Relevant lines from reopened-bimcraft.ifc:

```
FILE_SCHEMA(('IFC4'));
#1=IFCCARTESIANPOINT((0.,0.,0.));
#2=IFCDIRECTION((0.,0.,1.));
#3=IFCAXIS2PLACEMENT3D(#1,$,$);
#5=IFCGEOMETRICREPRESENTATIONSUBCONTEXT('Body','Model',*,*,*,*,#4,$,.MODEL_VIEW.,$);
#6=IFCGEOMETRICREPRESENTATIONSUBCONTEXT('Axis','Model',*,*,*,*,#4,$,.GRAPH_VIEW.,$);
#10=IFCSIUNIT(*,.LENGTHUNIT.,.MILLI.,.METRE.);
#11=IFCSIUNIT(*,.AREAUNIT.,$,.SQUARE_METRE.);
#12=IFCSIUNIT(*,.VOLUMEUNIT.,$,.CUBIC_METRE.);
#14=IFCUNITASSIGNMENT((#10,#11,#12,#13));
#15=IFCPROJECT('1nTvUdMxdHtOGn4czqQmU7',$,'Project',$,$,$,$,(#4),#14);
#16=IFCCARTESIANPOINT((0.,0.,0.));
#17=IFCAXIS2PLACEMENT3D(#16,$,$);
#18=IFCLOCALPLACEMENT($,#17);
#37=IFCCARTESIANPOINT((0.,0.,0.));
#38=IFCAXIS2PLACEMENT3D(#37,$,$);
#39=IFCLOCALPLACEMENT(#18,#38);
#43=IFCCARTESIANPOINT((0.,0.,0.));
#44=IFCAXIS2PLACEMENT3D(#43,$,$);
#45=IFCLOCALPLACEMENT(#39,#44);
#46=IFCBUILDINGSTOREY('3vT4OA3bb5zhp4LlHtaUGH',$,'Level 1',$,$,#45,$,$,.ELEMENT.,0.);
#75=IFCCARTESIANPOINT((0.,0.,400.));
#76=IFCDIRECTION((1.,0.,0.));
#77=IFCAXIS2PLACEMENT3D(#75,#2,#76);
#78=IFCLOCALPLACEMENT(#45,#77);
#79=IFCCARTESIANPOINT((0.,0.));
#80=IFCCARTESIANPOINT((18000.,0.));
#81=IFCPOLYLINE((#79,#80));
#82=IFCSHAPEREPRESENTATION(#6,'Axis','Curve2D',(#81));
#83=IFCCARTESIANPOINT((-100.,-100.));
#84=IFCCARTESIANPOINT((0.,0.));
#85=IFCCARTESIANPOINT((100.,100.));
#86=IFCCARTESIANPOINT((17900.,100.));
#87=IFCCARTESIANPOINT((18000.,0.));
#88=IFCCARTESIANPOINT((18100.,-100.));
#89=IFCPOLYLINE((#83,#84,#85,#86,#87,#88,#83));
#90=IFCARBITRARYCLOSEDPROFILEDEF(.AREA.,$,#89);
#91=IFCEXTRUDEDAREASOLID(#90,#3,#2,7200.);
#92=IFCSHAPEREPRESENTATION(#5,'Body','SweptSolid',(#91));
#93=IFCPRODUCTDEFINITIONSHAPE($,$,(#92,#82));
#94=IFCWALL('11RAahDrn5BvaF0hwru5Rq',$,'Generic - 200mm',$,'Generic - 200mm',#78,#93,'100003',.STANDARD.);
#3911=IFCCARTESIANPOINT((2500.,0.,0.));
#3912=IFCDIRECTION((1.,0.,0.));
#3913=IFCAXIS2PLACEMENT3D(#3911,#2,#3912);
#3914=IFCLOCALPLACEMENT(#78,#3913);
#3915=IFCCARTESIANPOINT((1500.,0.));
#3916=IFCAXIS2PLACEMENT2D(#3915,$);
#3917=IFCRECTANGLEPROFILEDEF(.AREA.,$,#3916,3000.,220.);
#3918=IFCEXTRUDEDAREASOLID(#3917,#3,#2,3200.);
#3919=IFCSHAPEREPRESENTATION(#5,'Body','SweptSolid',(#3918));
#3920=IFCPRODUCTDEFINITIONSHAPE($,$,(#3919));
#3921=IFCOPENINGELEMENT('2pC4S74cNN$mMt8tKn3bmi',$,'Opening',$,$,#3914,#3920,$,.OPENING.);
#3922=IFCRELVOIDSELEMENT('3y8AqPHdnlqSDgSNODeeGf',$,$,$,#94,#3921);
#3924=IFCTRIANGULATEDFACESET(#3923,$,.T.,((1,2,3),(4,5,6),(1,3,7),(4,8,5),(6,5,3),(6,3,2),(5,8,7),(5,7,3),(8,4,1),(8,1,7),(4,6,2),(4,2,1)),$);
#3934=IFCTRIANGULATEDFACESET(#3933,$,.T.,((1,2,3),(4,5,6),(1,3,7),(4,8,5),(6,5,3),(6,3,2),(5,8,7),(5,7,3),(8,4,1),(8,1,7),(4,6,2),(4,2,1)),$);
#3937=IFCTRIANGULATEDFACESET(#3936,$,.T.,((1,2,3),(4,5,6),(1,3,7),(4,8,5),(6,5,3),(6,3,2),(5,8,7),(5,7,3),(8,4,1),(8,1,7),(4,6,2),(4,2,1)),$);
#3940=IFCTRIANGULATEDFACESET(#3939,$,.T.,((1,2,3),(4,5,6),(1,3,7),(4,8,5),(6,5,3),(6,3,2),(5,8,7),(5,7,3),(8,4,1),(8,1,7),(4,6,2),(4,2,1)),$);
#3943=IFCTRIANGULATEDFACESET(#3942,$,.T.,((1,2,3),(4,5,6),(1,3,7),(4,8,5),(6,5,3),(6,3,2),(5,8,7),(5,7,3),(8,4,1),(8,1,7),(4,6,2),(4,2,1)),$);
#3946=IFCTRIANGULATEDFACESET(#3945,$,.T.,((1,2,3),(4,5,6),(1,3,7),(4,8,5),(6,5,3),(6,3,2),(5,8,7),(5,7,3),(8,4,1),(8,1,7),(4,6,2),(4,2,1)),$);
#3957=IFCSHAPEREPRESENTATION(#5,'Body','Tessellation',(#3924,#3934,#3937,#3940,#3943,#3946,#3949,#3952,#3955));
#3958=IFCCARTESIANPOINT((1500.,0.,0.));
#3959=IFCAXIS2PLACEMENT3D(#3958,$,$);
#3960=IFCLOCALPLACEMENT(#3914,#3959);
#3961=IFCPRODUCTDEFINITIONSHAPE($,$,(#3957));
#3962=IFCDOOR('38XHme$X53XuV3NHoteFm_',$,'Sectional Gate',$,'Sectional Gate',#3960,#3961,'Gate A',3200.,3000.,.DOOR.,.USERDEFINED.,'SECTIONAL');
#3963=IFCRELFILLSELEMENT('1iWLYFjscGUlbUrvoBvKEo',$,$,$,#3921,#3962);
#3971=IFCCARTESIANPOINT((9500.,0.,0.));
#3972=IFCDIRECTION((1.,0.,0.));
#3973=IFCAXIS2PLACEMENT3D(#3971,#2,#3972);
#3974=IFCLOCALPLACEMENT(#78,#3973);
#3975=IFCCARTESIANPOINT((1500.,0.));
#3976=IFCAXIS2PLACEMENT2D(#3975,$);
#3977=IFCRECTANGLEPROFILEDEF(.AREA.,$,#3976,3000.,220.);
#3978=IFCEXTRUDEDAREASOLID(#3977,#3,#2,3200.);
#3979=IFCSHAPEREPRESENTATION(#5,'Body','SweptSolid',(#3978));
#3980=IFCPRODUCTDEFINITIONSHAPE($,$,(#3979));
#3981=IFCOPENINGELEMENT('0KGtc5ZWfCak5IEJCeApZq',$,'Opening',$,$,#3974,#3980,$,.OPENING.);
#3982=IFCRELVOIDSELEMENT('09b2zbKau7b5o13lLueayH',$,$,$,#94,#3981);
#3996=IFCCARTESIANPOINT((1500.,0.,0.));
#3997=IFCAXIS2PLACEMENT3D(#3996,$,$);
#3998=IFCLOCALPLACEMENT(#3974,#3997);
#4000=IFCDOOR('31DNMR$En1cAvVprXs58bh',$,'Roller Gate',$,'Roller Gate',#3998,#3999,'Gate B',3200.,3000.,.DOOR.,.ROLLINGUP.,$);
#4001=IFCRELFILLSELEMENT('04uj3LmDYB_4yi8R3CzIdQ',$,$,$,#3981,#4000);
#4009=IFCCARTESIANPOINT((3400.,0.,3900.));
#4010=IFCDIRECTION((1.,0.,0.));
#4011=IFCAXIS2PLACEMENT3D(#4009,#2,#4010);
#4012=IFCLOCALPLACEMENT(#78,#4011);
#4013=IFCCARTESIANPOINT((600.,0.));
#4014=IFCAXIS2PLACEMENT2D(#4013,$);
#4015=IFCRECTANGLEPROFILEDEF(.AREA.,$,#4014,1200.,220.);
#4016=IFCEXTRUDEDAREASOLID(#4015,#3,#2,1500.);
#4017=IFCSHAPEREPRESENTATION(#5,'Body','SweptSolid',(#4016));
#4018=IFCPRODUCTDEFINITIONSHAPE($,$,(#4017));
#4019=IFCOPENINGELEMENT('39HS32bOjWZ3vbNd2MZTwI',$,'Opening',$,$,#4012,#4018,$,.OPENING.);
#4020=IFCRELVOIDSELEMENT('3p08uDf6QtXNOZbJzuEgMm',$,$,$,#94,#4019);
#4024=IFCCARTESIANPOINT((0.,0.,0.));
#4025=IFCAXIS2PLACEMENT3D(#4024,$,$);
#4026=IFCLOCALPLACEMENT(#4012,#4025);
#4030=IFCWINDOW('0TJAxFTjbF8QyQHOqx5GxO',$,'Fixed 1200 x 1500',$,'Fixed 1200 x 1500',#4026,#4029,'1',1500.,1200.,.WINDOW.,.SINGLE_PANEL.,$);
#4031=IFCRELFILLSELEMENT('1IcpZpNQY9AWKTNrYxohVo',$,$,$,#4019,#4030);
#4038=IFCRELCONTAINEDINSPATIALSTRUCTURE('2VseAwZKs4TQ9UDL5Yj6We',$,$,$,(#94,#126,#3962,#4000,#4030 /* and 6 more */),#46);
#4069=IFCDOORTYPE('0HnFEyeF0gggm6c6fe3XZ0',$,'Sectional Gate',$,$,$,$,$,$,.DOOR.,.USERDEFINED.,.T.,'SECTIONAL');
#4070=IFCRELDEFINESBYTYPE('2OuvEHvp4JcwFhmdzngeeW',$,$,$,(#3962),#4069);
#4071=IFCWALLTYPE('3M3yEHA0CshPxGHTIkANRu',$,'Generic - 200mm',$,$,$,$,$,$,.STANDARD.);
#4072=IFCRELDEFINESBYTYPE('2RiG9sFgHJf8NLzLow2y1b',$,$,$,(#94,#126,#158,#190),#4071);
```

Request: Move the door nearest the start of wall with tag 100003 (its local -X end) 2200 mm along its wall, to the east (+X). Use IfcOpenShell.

```python
import ifcopenshell
import ifcopenshell.api.geometry
import ifcopenshell.util.placement
import ifcopenshell.util.unit

model = ifcopenshell.open("reopened-bimcraft.ifc")
unit_scale = ifcopenshell.util.unit.calculate_unit_scale(model)

door = model.by_guid("38XHme$X53XuV3NHoteFm_")
opening = door.FillsVoids[0].RelatingOpeningElement
wall = opening.VoidsElements[0].RelatingBuildingElement

wall_matrix = ifcopenshell.util.placement.get_local_placement(wall.ObjectPlacement)
shift = wall_matrix[:3, 0] * 2.2 / unit_scale
before = ifcopenshell.util.placement.get_local_placement(door.ObjectPlacement)[:3, 3].copy()

# The door is placed relative to its opening, so it follows when the opening moves.
matrix = ifcopenshell.util.placement.get_local_placement(opening.ObjectPlacement)
matrix[:3, 3] += shift
ifcopenshell.api.geometry.edit_object_placement(
    model, product=opening, matrix=matrix, is_si=False, should_transform_children=True
)

after = ifcopenshell.util.placement.get_local_placement(door.ObjectPlacement)[:3, 3]
print("door moved by", (after - before).round(3) + 0.0)

model.write("reopened-bimcraft_v2.ifc")
```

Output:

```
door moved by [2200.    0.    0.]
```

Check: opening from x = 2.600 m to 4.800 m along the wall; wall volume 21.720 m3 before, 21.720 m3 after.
